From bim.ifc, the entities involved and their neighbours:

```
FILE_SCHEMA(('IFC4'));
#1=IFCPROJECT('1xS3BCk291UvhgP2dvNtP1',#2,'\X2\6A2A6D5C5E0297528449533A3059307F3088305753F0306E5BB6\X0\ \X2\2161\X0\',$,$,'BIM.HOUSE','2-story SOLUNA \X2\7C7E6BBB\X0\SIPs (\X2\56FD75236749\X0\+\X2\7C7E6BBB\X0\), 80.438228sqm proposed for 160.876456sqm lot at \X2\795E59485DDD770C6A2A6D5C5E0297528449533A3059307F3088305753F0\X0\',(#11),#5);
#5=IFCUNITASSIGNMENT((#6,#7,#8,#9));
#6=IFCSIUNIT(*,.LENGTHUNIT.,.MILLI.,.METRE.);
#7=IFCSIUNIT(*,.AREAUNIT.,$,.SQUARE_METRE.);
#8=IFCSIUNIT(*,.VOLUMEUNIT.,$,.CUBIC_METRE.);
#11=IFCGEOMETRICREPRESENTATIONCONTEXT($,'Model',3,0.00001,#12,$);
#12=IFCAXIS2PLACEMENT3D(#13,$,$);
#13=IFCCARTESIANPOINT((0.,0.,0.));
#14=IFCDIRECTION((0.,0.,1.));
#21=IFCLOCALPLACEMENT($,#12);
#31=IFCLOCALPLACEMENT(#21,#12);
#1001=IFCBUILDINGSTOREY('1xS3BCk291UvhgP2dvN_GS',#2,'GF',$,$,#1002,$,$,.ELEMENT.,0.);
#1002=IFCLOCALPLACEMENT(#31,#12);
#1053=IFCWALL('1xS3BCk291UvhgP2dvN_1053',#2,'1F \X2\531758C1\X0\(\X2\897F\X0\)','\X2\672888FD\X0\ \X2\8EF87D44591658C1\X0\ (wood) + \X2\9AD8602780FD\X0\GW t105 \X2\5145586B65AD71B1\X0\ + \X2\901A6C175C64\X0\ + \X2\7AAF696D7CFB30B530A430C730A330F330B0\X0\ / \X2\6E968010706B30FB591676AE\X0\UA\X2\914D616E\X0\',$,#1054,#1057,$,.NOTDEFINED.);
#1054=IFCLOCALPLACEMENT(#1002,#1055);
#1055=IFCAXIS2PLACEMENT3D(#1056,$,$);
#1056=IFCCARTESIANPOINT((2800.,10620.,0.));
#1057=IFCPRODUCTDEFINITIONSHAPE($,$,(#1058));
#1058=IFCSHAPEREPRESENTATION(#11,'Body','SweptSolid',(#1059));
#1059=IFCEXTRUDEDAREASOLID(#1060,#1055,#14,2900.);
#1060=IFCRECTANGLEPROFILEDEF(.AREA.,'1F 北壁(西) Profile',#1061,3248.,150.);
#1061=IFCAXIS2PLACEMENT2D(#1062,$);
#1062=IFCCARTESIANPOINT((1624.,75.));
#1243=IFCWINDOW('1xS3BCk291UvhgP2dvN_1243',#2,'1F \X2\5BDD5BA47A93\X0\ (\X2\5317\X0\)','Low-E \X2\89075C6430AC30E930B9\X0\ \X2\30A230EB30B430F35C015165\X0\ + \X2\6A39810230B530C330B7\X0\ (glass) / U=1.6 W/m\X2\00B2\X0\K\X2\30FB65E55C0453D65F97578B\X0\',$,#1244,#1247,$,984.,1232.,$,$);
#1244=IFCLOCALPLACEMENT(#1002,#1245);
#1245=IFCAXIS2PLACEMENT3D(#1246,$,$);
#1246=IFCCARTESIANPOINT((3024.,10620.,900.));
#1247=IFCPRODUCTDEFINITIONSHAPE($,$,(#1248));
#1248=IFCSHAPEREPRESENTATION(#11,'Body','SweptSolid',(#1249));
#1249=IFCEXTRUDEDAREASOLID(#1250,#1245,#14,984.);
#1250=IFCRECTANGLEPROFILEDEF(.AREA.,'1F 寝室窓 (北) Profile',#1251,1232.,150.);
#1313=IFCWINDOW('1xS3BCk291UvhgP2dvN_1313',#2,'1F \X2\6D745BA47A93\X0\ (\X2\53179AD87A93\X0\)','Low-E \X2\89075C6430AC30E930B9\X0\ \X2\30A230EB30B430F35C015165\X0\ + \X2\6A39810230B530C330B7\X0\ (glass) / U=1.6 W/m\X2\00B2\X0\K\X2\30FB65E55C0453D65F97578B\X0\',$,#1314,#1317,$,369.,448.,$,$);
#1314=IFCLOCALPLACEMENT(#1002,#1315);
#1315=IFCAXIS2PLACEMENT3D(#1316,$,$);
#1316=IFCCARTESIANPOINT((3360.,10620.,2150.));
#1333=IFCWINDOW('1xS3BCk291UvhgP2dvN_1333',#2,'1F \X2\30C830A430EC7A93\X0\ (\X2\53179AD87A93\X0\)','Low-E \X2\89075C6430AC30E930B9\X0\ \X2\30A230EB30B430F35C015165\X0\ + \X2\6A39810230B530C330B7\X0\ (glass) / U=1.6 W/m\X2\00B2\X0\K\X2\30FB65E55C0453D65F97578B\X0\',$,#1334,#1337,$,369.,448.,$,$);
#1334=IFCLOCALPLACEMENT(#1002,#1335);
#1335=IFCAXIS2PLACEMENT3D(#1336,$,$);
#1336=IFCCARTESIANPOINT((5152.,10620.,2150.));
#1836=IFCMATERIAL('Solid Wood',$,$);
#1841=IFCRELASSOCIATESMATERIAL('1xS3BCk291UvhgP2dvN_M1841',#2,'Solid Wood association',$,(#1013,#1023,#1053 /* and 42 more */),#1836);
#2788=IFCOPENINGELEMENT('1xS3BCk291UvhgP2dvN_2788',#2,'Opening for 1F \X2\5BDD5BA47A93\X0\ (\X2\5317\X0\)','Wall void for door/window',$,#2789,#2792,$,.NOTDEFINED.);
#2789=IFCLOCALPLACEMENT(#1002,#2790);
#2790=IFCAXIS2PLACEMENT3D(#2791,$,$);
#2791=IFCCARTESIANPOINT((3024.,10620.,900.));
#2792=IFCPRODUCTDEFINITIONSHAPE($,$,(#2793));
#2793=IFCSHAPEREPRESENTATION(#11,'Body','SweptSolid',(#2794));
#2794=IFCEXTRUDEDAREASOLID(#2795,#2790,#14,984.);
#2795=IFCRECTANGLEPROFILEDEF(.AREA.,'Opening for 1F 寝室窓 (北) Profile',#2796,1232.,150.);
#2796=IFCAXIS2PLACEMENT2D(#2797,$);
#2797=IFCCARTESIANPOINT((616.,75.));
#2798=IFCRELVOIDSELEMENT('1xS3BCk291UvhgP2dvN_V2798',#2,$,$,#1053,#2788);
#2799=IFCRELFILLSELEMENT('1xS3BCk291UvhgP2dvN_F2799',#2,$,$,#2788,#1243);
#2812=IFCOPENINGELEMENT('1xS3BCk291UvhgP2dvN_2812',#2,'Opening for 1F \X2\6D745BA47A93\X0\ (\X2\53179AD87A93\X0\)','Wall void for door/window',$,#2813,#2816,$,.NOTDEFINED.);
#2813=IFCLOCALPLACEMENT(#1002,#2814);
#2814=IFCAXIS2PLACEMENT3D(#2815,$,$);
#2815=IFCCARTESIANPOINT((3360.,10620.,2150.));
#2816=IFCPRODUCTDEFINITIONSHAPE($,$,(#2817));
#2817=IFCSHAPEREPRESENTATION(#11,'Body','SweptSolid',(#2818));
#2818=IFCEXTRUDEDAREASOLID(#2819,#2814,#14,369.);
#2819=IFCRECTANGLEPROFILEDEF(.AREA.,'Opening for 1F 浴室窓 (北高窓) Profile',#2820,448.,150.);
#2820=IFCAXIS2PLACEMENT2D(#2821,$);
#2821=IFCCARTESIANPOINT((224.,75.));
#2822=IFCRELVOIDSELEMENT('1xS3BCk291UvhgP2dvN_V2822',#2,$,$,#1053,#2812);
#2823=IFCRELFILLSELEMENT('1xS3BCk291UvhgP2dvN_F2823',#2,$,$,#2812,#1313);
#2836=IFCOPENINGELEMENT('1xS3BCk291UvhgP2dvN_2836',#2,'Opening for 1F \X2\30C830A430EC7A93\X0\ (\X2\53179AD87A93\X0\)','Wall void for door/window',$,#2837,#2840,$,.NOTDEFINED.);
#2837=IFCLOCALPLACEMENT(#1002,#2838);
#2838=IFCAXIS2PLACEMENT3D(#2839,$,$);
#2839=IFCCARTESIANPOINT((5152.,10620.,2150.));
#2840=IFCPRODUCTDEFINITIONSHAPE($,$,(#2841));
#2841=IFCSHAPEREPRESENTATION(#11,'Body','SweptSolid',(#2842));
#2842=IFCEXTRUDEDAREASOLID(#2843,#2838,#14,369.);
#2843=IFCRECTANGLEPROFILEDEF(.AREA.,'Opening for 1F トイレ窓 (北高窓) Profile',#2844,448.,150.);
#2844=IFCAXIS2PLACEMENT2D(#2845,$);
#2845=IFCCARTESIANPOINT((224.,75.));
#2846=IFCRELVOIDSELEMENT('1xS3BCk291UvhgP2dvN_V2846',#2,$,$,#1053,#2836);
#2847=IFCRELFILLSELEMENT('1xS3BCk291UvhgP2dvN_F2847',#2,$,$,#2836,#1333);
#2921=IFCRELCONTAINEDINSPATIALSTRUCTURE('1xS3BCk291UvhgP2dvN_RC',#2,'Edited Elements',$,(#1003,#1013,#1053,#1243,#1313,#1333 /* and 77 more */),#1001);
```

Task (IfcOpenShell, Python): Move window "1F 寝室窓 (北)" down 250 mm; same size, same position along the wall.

```python
import numpy as np
import ifcopenshell
import ifcopenshell.api.geometry
import ifcopenshell.util.placement
import ifcopenshell.util.unit

model = ifcopenshell.open("bim.ifc")
unit_scale = ifcopenshell.util.unit.calculate_unit_scale(model)

window = model.by_id(1243)
opening = window.FillsVoids[0].RelatingOpeningElement
dz = -0.25 / unit_scale

shift = np.array([0.0, 0.0, dz])
# The window is not placed relative to its opening, so move both.
for product in (opening, window):
    matrix = ifcopenshell.util.placement.get_local_placement(product.ObjectPlacement)
    matrix[:3, 3] += shift
    ifcopenshell.api.geometry.edit_object_placement(model, product=product, matrix=matrix, is_si=False)

print(f"moved by {dz * unit_scale:+.3f} m")

model.write("bim_edited.ifc")
```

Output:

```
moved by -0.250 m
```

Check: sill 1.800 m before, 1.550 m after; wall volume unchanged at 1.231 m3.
